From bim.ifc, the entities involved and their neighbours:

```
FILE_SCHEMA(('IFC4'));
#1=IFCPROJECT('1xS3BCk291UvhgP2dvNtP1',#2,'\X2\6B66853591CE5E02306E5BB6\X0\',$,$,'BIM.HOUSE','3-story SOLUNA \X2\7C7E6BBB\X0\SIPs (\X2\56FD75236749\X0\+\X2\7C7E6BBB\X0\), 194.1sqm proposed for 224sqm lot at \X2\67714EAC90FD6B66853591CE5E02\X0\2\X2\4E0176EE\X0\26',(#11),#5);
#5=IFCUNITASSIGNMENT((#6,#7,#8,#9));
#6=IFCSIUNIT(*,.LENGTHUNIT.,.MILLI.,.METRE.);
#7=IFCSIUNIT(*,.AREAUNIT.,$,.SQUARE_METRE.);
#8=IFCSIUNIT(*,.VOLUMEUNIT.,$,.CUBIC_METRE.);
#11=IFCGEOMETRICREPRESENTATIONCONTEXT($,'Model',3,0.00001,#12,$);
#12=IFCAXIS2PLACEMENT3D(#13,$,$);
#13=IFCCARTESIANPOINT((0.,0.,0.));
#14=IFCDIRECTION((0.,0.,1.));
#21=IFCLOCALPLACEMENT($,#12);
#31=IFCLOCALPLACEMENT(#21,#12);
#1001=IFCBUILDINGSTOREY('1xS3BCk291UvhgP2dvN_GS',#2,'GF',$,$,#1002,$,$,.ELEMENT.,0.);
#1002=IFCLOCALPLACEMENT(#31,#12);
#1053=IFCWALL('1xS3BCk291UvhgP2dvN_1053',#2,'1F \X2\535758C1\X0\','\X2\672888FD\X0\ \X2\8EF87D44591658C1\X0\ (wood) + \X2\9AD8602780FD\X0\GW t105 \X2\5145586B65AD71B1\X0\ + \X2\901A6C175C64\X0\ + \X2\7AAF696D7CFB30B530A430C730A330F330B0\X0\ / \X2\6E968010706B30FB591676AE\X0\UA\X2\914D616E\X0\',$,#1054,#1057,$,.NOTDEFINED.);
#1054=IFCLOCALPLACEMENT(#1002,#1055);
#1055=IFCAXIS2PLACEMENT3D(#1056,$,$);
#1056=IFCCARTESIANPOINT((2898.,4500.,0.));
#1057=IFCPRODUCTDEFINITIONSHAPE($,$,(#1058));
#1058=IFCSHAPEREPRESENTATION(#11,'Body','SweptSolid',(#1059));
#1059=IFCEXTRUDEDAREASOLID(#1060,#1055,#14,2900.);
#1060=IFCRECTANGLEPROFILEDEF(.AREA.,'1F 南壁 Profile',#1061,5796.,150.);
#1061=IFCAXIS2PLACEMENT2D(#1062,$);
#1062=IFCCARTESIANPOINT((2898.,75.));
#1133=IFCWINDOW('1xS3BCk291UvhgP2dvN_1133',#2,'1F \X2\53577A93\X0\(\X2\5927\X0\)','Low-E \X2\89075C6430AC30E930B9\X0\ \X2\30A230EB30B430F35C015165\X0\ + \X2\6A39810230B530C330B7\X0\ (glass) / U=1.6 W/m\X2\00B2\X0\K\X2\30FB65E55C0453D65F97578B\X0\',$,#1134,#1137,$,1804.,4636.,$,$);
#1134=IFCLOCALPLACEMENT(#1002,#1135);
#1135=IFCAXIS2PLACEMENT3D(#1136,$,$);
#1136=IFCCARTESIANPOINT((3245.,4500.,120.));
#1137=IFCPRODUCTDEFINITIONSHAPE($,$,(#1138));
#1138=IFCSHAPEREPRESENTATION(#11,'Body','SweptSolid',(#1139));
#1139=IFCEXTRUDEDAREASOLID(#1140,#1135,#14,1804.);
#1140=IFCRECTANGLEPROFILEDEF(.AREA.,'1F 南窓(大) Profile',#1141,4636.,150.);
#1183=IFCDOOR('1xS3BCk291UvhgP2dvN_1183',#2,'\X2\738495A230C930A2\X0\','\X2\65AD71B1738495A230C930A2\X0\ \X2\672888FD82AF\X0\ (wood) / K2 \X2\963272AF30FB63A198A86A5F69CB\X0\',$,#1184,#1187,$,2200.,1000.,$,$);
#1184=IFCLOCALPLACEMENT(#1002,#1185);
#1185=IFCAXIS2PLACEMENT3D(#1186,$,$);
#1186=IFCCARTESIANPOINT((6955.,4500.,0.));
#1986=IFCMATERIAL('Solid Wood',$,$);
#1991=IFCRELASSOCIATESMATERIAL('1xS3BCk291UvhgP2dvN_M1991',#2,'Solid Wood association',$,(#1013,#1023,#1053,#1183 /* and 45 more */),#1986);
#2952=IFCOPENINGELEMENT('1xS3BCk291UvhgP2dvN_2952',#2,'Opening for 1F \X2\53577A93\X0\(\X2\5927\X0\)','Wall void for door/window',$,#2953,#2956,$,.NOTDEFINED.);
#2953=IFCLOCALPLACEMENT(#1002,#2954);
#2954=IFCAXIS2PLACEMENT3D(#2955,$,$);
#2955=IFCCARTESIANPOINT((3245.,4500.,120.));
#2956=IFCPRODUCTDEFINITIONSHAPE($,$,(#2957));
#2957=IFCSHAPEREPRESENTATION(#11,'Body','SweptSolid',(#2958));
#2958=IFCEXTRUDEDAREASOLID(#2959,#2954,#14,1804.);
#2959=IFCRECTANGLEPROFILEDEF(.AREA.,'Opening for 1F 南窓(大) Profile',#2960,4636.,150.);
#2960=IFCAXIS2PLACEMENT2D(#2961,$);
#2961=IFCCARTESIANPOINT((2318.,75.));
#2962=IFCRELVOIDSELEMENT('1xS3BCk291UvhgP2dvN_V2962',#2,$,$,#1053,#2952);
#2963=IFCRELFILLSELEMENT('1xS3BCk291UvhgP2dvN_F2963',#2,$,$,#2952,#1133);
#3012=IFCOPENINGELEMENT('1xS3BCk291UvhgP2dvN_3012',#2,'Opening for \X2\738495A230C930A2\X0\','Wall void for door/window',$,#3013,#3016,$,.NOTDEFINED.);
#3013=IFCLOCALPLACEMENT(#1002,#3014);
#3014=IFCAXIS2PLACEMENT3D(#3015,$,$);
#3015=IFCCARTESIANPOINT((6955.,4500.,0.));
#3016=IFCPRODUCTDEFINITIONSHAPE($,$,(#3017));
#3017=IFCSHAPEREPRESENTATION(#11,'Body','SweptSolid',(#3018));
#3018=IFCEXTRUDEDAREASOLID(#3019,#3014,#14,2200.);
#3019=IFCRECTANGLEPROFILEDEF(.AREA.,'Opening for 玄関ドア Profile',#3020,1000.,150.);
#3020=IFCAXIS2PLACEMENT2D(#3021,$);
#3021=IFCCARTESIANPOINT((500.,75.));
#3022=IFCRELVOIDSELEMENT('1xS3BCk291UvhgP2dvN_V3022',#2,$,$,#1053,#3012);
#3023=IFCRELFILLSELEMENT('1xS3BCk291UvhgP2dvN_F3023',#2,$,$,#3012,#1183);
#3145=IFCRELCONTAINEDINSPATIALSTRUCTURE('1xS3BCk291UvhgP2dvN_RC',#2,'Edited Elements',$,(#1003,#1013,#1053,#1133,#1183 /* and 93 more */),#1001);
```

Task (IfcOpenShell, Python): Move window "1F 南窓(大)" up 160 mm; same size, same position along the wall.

```python
import numpy as np
import ifcopenshell
import ifcopenshell.api.geometry
import ifcopenshell.util.placement
import ifcopenshell.util.unit

model = ifcopenshell.open("bim.ifc")
unit_scale = ifcopenshell.util.unit.calculate_unit_scale(model)

window = model.by_guid("1xS3BCk291UvhgP2dvN_1133")
opening = window.FillsVoids[0].RelatingOpeningElement
dz = 0.16 / unit_scale

shift = np.array([0.0, 0.0, dz])
# The window is not placed relative to its opening, so move both.
for product in (opening, window):
    matrix = ifcopenshell.util.placement.get_local_placement(product.ObjectPlacement)
    matrix[:3, 3] += shift
    ifcopenshell.api.geometry.edit_object_placement(model, product=product, matrix=matrix, is_si=False)

print(f"moved by {dz * unit_scale:+.3f} m")

model.write("bim_v2.ifc")
```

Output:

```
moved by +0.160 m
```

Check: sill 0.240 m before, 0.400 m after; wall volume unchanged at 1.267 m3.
